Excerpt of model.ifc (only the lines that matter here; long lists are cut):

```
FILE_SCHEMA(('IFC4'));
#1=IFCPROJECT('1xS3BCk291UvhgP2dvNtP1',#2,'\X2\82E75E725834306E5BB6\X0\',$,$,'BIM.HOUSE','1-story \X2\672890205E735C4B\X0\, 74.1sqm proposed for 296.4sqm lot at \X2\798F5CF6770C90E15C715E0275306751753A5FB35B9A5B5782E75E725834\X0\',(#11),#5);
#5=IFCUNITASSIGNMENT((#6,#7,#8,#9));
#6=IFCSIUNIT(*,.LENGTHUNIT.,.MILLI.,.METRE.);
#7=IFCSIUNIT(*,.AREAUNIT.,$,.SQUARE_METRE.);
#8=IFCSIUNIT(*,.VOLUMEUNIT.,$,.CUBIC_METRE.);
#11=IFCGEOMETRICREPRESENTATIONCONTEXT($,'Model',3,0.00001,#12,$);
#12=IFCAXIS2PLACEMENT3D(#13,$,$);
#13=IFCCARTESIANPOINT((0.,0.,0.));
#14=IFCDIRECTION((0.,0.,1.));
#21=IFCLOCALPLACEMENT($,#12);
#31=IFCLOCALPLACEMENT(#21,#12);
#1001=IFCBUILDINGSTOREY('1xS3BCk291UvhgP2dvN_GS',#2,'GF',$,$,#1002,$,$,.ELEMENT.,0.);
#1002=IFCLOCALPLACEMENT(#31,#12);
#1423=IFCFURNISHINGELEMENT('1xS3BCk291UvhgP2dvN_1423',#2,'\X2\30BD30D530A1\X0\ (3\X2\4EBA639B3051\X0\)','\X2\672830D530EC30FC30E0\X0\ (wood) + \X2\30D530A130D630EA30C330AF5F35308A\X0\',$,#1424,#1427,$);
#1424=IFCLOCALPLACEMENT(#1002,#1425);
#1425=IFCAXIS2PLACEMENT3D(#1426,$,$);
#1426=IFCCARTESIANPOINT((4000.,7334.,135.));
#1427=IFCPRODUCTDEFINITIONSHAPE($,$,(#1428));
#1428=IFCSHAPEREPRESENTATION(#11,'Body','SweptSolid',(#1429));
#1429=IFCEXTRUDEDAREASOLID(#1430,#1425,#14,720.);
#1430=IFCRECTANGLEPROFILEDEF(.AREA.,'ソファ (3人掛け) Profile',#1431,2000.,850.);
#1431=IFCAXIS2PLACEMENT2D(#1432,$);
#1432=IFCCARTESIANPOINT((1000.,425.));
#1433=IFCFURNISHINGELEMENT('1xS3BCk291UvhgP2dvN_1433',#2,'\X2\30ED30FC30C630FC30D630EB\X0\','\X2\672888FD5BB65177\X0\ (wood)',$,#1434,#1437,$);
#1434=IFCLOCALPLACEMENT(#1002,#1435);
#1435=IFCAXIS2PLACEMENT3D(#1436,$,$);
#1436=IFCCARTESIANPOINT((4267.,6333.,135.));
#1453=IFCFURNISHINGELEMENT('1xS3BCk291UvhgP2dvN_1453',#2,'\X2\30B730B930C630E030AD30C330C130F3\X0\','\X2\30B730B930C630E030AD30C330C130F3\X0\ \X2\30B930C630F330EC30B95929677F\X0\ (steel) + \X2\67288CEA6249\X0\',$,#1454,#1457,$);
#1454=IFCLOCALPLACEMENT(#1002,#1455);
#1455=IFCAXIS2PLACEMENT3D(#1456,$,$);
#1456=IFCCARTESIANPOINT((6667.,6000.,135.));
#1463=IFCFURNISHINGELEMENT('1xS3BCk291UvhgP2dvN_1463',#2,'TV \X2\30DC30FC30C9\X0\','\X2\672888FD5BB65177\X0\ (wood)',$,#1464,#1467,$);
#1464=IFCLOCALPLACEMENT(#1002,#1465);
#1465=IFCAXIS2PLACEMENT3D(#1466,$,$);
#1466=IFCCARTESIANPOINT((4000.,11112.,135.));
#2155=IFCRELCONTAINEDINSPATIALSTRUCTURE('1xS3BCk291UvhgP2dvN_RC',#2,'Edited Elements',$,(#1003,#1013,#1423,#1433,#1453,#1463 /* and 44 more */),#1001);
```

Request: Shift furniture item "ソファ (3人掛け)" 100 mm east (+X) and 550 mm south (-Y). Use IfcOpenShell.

```python
import ifcopenshell
import ifcopenshell.api.geometry
import ifcopenshell.util.placement
import ifcopenshell.util.unit

model = ifcopenshell.open("model.ifc")
unit_scale = ifcopenshell.util.unit.calculate_unit_scale(model)

item = model.by_guid("1xS3BCk291UvhgP2dvN_1423")
matrix = ifcopenshell.util.placement.get_local_placement(item.ObjectPlacement)
matrix[0, 3] += 0.1 / unit_scale
matrix[1, 3] -= 0.55 / unit_scale
ifcopenshell.api.geometry.edit_object_placement(model, product=item, matrix=matrix, is_si=False)

print(ifcopenshell.util.placement.get_local_placement(item.ObjectPlacement).round(3) + 0.0)

model.write("model_rev.ifc")
```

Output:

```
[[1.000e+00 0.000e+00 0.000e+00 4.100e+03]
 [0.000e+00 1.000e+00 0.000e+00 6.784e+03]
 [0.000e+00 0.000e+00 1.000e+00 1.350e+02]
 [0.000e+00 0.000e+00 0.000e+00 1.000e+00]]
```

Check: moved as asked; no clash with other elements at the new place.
